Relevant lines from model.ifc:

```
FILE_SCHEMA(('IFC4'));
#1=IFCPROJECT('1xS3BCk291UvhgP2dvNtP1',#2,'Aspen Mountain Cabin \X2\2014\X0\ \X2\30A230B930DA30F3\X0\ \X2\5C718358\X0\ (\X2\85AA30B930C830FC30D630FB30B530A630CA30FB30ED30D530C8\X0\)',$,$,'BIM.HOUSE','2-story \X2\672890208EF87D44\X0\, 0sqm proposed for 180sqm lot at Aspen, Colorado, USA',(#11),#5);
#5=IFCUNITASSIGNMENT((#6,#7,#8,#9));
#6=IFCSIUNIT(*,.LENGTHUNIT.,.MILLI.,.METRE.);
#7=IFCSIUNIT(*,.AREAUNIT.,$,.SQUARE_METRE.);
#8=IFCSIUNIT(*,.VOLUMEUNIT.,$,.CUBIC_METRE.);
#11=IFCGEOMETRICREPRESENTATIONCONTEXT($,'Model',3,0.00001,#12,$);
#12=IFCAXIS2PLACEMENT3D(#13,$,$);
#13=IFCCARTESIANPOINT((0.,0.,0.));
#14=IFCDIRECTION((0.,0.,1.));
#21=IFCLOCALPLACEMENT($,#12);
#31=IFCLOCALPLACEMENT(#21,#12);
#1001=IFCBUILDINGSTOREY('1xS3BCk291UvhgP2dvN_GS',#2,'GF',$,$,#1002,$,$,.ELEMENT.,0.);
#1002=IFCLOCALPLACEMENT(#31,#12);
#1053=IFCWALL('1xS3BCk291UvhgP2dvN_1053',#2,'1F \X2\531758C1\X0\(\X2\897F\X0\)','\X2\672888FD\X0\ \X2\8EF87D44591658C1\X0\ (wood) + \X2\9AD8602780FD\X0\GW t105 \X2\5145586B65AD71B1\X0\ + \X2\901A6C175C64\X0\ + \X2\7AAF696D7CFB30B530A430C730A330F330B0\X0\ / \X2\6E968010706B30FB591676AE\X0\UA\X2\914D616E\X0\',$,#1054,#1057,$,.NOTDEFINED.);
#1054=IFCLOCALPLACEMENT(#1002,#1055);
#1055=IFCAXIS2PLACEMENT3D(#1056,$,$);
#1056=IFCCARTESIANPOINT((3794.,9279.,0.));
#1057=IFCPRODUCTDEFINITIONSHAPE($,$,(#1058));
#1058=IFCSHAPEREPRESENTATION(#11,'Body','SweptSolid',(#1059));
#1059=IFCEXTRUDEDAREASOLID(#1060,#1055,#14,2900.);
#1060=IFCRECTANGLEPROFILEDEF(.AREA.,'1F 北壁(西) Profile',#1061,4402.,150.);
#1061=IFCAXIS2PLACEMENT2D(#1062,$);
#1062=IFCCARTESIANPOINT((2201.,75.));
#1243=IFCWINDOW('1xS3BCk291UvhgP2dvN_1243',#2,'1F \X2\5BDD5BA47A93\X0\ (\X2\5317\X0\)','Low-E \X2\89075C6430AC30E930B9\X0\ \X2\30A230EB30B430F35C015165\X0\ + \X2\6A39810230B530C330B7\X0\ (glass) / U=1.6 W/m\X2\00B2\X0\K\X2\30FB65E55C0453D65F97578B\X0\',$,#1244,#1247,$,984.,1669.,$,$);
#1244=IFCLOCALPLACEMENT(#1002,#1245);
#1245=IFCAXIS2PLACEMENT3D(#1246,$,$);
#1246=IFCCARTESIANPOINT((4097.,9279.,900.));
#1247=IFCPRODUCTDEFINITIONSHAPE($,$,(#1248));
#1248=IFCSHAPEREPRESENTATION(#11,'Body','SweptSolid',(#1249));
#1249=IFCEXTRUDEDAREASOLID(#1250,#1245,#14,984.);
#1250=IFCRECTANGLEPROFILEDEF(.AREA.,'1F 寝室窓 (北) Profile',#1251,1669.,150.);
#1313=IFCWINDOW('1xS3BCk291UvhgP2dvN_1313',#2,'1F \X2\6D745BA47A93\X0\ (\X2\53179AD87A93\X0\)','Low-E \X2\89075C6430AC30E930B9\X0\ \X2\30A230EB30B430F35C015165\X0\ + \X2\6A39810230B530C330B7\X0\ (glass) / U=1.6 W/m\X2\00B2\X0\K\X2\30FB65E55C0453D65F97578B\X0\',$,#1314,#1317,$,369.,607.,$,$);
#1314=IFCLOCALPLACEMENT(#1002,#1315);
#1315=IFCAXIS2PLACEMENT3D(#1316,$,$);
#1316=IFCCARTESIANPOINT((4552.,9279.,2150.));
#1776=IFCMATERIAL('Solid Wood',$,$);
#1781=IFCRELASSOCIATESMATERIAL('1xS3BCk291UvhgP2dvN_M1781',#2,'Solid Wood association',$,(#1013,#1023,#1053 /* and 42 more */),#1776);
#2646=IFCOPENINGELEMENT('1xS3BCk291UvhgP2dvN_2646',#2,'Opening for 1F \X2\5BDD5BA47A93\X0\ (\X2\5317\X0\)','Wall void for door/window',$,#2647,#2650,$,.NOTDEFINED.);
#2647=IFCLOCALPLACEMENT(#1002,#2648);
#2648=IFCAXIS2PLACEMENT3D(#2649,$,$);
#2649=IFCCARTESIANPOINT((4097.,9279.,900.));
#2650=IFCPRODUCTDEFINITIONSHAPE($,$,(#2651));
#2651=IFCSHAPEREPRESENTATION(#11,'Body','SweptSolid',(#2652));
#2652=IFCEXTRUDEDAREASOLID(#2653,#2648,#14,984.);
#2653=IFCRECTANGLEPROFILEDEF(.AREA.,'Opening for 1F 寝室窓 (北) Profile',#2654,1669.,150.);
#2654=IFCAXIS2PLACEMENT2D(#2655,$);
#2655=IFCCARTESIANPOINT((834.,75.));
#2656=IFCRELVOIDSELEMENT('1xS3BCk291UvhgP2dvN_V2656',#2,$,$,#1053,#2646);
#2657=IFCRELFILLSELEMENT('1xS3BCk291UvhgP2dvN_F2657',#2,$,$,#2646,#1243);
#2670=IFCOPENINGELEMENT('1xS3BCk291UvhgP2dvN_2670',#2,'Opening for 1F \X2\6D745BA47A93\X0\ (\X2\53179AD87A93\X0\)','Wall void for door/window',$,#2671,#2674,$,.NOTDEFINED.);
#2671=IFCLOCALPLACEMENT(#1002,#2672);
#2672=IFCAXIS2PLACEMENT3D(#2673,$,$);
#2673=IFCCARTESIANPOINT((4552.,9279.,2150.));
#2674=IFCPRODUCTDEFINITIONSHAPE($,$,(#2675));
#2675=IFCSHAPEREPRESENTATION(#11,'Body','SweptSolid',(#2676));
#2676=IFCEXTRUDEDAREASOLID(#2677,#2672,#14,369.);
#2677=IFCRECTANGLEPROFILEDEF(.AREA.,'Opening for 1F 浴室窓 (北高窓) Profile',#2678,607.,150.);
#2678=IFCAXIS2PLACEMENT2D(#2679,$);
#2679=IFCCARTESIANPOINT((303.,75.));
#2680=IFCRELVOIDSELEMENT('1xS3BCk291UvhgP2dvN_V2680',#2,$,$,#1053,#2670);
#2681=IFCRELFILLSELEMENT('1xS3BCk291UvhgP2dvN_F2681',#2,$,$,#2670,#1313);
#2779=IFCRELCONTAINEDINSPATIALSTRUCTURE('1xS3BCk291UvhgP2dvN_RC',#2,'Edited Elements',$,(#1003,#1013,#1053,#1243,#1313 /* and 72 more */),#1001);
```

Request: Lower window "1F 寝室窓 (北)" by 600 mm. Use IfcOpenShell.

```python
import numpy as np
import ifcopenshell
import ifcopenshell.api.geometry
import ifcopenshell.util.placement
import ifcopenshell.util.unit

model = ifcopenshell.open("model.ifc")
unit_scale = ifcopenshell.util.unit.calculate_unit_scale(model)

window = model.by_id(1243)
opening = window.FillsVoids[0].RelatingOpeningElement
dz = -0.6 / unit_scale

shift = np.array([0.0, 0.0, dz])
# The window is not placed relative to its opening, so move both.
for product in (opening, window):
    matrix = ifcopenshell.util.placement.get_local_placement(product.ObjectPlacement)
    matrix[:3, 3] += shift
    ifcopenshell.api.geometry.edit_object_placement(model, product=product, matrix=matrix, is_si=False)

print(f"moved by {dz * unit_scale:+.3f} m")

model.write("model_v2.ifc")
```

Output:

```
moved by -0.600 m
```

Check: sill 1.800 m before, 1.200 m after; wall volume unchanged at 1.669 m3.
